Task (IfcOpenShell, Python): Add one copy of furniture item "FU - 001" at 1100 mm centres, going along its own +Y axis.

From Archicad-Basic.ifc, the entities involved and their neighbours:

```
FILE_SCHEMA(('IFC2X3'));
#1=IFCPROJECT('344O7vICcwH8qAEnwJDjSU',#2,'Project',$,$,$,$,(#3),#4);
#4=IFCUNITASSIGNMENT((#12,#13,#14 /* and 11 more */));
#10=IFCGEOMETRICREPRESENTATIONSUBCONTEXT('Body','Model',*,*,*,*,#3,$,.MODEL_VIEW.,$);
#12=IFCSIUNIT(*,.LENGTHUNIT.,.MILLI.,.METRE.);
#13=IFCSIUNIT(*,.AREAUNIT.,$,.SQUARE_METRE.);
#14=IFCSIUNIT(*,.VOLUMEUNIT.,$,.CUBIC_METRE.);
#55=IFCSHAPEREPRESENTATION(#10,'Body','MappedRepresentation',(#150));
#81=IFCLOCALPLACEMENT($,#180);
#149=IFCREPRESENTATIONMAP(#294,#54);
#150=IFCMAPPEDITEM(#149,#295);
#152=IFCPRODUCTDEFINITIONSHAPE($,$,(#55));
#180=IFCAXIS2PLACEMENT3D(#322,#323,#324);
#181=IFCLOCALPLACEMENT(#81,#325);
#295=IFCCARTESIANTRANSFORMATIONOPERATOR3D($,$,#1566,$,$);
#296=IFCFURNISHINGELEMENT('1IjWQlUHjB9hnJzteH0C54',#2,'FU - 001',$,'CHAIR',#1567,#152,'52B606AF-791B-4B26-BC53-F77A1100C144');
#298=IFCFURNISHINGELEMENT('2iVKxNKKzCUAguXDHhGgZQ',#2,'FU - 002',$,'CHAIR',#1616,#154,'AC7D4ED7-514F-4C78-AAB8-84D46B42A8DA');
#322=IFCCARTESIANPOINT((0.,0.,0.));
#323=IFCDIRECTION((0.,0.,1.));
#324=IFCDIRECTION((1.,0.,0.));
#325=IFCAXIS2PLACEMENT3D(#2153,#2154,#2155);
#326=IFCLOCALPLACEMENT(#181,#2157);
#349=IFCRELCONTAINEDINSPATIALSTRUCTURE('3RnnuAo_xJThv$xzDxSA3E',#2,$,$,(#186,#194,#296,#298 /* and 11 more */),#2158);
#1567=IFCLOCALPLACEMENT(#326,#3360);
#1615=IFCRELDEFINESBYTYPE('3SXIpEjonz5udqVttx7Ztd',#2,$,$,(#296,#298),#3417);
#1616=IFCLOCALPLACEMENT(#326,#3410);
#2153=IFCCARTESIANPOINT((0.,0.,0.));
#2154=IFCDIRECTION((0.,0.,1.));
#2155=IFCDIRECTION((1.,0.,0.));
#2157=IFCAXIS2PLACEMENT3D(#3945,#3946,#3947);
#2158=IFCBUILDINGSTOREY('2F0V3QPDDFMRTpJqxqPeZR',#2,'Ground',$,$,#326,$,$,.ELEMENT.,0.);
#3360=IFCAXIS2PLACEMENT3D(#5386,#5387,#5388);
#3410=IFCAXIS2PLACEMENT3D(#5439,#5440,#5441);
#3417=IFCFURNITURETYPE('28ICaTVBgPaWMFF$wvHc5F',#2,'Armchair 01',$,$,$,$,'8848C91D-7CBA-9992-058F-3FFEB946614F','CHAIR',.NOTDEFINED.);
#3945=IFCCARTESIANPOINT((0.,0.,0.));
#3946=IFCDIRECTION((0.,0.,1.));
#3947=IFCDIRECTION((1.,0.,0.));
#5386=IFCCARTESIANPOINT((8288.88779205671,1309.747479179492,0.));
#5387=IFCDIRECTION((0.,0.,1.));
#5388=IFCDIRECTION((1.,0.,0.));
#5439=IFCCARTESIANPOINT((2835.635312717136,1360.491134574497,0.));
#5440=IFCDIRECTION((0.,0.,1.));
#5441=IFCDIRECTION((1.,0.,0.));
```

```python
import ifcopenshell
import ifcopenshell.api.geometry
import ifcopenshell.api.root
import ifcopenshell.util.element
import ifcopenshell.util.placement

model = ifcopenshell.open("Archicad-Basic.ifc")


def reuse_history(source, copy):
    """copy_class also copies each property set's owner history, people and application; keep the originals."""
    for rel in copy.IsDefinedBy:
        if rel.is_a("IfcRelDefinesByProperties") and (history := rel.RelatingPropertyDefinition.OwnerHistory):
            rel.RelatingPropertyDefinition.OwnerHistory = source.OwnerHistory
            ifcopenshell.util.element.remove_deep2(model, history)


source = model.by_guid("1IjWQlUHjB9hnJzteH0C54")
base = ifcopenshell.util.placement.get_local_placement(source.ObjectPlacement)
step = base[:3, 1] * 1100.0

for i in range(1, 2):
    copy = ifcopenshell.api.root.copy_class(model, product=source)
    copy.Representation = ifcopenshell.util.element.copy_deep(
        model, source.Representation, exclude=["IfcGeometricRepresentationContext", "IfcRepresentationMap"]
    )
    copy.Tag = None
    reuse_history(source, copy)
    matrix = base.copy()
    matrix[:3, 3] += i * step
    print("added at", matrix[:3, 3].round(3) + 0.0)
    ifcopenshell.api.geometry.edit_object_placement(model, product=copy, matrix=matrix, is_si=False)

model.write("Archicad-Basic_edited.ifc")
```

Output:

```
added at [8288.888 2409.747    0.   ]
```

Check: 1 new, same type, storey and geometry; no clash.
